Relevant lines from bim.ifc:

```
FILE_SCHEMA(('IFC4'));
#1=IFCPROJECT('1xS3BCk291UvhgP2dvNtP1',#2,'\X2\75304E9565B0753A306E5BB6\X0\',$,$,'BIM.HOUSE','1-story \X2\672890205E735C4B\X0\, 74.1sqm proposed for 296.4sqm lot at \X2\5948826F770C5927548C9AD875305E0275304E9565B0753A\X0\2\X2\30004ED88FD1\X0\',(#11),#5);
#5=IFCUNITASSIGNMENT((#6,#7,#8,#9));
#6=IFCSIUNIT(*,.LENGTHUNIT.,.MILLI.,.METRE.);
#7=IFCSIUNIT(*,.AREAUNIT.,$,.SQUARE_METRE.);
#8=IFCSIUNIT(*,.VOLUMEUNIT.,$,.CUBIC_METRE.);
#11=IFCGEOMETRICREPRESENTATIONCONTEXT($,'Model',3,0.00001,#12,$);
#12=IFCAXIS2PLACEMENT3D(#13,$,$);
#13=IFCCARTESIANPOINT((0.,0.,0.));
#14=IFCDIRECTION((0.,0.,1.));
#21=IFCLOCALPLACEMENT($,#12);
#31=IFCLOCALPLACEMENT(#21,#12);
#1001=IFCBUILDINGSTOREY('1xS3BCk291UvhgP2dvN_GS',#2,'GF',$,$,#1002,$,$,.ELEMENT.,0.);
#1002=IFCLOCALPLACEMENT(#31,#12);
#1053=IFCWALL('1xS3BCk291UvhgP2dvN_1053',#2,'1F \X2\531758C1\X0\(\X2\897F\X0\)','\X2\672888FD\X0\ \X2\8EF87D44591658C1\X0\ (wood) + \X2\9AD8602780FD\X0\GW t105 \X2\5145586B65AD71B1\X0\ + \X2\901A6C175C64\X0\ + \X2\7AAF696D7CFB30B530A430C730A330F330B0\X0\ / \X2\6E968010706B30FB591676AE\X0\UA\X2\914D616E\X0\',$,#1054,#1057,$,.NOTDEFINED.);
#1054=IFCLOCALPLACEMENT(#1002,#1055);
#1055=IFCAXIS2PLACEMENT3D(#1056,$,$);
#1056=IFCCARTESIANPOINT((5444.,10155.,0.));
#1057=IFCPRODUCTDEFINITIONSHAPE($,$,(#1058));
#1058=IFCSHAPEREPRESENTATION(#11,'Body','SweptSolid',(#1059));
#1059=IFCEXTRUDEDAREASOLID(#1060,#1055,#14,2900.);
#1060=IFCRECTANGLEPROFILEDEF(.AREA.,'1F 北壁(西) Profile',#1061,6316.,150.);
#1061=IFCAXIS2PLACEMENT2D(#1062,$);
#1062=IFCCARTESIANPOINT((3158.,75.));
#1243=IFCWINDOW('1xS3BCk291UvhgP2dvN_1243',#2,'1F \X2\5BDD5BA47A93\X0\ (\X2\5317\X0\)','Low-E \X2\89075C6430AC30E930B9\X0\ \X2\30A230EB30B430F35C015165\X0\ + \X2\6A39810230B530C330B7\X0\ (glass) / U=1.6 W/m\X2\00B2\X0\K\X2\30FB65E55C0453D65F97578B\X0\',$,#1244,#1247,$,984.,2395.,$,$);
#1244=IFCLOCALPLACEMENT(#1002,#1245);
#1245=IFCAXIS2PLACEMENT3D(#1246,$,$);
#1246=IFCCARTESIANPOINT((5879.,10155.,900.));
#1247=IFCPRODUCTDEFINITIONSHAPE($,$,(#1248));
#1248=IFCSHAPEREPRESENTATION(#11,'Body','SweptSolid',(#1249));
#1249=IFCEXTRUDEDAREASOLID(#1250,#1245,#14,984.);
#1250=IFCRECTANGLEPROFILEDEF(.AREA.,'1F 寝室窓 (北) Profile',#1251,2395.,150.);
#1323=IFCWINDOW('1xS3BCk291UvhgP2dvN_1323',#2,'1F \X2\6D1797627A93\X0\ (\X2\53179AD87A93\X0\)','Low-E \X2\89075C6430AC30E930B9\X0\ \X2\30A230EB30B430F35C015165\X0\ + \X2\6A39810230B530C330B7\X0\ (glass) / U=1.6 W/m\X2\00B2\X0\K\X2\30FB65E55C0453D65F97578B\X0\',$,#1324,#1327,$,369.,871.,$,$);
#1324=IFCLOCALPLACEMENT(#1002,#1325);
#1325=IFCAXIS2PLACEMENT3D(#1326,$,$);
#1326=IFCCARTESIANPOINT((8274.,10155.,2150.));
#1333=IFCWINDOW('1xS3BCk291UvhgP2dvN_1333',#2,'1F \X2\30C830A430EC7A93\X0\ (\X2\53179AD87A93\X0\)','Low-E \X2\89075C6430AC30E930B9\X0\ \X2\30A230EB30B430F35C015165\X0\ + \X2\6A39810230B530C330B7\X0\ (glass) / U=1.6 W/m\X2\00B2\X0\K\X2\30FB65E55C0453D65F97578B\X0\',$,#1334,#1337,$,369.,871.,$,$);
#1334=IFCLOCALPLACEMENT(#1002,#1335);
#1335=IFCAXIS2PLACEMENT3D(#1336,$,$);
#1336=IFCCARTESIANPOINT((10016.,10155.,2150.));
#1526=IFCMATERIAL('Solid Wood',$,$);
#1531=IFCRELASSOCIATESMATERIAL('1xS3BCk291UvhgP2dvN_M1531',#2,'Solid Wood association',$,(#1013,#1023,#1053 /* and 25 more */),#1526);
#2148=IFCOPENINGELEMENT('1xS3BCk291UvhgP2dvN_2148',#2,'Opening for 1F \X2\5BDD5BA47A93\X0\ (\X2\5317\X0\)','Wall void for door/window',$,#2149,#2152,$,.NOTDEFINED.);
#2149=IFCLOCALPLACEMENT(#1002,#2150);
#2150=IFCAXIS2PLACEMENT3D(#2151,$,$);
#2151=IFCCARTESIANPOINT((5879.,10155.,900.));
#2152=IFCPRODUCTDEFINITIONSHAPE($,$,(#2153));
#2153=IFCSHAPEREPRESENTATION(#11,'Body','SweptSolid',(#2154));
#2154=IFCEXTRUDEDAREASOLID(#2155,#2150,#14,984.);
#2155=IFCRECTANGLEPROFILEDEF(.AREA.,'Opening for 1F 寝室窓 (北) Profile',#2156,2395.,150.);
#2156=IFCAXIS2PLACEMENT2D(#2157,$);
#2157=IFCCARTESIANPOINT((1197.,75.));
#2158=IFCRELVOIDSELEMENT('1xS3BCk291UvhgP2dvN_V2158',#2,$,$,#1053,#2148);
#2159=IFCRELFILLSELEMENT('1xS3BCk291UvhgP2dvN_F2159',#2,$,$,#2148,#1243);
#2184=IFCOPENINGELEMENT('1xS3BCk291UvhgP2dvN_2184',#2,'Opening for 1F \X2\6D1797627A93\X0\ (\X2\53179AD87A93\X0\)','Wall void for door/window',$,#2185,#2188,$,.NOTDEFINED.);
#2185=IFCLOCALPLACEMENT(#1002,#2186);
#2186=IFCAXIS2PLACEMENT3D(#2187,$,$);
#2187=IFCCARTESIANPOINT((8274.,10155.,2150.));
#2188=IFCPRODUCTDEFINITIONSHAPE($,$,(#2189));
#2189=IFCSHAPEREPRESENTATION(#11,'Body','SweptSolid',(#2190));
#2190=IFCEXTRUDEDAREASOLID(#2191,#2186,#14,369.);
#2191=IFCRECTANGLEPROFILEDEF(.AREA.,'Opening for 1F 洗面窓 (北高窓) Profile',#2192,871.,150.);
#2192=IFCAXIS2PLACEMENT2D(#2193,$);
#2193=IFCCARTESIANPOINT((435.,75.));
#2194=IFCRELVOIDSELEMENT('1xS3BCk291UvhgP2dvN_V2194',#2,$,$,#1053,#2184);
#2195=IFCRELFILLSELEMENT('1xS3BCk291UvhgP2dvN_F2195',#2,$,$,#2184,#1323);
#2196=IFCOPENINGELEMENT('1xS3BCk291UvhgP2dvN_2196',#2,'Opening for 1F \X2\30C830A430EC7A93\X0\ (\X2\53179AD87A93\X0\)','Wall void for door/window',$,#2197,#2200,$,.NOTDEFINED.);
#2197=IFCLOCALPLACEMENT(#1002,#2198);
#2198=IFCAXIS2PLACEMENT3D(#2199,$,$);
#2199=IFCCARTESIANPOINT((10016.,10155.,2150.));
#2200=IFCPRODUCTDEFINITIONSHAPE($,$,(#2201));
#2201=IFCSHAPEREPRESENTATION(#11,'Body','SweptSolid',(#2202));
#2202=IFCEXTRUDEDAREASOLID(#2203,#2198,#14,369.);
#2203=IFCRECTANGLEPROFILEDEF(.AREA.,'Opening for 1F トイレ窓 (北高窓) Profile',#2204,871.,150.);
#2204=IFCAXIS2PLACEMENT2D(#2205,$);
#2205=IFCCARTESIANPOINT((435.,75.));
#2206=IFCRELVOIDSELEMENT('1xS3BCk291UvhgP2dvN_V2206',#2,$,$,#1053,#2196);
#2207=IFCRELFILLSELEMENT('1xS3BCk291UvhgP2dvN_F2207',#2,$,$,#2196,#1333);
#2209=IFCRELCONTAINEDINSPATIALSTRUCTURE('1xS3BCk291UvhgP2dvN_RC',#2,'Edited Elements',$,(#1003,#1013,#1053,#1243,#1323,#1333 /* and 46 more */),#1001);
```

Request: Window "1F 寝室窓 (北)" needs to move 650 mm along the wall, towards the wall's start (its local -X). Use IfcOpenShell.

```python
import ifcopenshell
import ifcopenshell.api.geometry
import ifcopenshell.util.placement
import ifcopenshell.util.unit

model = ifcopenshell.open("bim.ifc")
unit_scale = ifcopenshell.util.unit.calculate_unit_scale(model)

window = model.by_guid("1xS3BCk291UvhgP2dvN_1243")
opening = window.FillsVoids[0].RelatingOpeningElement
wall = opening.VoidsElements[0].RelatingBuildingElement

wall_matrix = ifcopenshell.util.placement.get_local_placement(wall.ObjectPlacement)
shift = wall_matrix[:3, 0] * -0.65 / unit_scale
before = ifcopenshell.util.placement.get_local_placement(window.ObjectPlacement)[:3, 3].copy()

# The window is not placed relative to its opening, so move both.
for product in (opening, window):
    matrix = ifcopenshell.util.placement.get_local_placement(product.ObjectPlacement)
    matrix[:3, 3] += shift
    ifcopenshell.api.geometry.edit_object_placement(model, product=product, matrix=matrix, is_si=False)

after = ifcopenshell.util.placement.get_local_placement(window.ObjectPlacement)[:3, 3]
print("window moved by", (after - before).round(3) + 0.0)

model.write("bim_v2.ifc")
```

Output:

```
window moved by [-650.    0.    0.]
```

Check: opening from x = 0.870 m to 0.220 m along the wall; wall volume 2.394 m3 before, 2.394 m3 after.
